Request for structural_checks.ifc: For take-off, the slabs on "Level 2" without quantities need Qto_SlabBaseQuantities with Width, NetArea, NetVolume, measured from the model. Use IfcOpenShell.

First a look at what the model holds.

```python
import ifcopenshell
import ifcopenshell.util.element
import ifcopenshell.util.unit

model = ifcopenshell.open("structural_checks.ifc")
print(model.schema)
for unit_type in ("LENGTHUNIT", "AREAUNIT", "VOLUMEUNIT"):
    print(unit_type, ifcopenshell.util.unit.calculate_unit_scale(model, unit_type))
storey = next(s for s in model.by_type("IfcBuildingStorey") if s.Name == "Level 2")
slabs = [e for e in ifcopenshell.util.element.get_decomposition(storey) if e.is_a("IfcSlab")]
for e in sorted(slabs, key=lambda e: e.id()):
    print(e.id(), e.is_a(), e.Name, list(ifcopenshell.util.element.get_psets(e, qtos_only=True)), sep=" | ")
```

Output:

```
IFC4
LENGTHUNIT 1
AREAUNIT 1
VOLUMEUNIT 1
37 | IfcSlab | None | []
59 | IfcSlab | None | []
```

```python
import ifcopenshell
import ifcopenshell.api.pset
import ifcopenshell.geom
import ifcopenshell.util.element
import ifcopenshell.util.shape
import ifcopenshell.util.unit

model = ifcopenshell.open("structural_checks.ifc")
unit_scale = ifcopenshell.util.unit.calculate_unit_scale(model)
area_scale = ifcopenshell.util.unit.calculate_unit_scale(model, "AREAUNIT")
volume_scale = ifcopenshell.util.unit.calculate_unit_scale(model, "VOLUMEUNIT")
settings = ifcopenshell.geom.settings()

storey = next(s for s in model.by_type("IfcBuildingStorey") if s.Name == "Level 2")
slabs = [e for e in ifcopenshell.util.element.get_decomposition(storey) if e.is_a("IfcSlab")]

for e in sorted(slabs, key=lambda e: e.id()):
    if ifcopenshell.util.element.get_psets(e, qtos_only=True, should_inherit=False):
        continue
    # Geometry comes back in metres, in the element's own axes.
    shape = ifcopenshell.geom.create_shape(settings, e)
    values = {
        "Width": ifcopenshell.util.shape.get_z(shape.geometry) / unit_scale,
        "NetArea": ifcopenshell.util.shape.get_footprint_area(shape.geometry) / area_scale,
        "NetVolume": ifcopenshell.util.shape.get_volume(shape.geometry) / volume_scale,
    }
    qto = ifcopenshell.api.pset.add_qto(model, product=e, name="Qto_SlabBaseQuantities")
    ifcopenshell.api.pset.edit_qto(model, qto=qto, properties=values)
    print(e.id(), {k: round(v, 3) for k, v in values.items()})

model.write("structural_checks_edited.ifc")
```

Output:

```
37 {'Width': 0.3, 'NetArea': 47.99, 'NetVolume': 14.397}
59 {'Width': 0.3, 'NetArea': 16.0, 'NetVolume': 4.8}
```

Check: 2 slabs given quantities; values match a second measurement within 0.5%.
